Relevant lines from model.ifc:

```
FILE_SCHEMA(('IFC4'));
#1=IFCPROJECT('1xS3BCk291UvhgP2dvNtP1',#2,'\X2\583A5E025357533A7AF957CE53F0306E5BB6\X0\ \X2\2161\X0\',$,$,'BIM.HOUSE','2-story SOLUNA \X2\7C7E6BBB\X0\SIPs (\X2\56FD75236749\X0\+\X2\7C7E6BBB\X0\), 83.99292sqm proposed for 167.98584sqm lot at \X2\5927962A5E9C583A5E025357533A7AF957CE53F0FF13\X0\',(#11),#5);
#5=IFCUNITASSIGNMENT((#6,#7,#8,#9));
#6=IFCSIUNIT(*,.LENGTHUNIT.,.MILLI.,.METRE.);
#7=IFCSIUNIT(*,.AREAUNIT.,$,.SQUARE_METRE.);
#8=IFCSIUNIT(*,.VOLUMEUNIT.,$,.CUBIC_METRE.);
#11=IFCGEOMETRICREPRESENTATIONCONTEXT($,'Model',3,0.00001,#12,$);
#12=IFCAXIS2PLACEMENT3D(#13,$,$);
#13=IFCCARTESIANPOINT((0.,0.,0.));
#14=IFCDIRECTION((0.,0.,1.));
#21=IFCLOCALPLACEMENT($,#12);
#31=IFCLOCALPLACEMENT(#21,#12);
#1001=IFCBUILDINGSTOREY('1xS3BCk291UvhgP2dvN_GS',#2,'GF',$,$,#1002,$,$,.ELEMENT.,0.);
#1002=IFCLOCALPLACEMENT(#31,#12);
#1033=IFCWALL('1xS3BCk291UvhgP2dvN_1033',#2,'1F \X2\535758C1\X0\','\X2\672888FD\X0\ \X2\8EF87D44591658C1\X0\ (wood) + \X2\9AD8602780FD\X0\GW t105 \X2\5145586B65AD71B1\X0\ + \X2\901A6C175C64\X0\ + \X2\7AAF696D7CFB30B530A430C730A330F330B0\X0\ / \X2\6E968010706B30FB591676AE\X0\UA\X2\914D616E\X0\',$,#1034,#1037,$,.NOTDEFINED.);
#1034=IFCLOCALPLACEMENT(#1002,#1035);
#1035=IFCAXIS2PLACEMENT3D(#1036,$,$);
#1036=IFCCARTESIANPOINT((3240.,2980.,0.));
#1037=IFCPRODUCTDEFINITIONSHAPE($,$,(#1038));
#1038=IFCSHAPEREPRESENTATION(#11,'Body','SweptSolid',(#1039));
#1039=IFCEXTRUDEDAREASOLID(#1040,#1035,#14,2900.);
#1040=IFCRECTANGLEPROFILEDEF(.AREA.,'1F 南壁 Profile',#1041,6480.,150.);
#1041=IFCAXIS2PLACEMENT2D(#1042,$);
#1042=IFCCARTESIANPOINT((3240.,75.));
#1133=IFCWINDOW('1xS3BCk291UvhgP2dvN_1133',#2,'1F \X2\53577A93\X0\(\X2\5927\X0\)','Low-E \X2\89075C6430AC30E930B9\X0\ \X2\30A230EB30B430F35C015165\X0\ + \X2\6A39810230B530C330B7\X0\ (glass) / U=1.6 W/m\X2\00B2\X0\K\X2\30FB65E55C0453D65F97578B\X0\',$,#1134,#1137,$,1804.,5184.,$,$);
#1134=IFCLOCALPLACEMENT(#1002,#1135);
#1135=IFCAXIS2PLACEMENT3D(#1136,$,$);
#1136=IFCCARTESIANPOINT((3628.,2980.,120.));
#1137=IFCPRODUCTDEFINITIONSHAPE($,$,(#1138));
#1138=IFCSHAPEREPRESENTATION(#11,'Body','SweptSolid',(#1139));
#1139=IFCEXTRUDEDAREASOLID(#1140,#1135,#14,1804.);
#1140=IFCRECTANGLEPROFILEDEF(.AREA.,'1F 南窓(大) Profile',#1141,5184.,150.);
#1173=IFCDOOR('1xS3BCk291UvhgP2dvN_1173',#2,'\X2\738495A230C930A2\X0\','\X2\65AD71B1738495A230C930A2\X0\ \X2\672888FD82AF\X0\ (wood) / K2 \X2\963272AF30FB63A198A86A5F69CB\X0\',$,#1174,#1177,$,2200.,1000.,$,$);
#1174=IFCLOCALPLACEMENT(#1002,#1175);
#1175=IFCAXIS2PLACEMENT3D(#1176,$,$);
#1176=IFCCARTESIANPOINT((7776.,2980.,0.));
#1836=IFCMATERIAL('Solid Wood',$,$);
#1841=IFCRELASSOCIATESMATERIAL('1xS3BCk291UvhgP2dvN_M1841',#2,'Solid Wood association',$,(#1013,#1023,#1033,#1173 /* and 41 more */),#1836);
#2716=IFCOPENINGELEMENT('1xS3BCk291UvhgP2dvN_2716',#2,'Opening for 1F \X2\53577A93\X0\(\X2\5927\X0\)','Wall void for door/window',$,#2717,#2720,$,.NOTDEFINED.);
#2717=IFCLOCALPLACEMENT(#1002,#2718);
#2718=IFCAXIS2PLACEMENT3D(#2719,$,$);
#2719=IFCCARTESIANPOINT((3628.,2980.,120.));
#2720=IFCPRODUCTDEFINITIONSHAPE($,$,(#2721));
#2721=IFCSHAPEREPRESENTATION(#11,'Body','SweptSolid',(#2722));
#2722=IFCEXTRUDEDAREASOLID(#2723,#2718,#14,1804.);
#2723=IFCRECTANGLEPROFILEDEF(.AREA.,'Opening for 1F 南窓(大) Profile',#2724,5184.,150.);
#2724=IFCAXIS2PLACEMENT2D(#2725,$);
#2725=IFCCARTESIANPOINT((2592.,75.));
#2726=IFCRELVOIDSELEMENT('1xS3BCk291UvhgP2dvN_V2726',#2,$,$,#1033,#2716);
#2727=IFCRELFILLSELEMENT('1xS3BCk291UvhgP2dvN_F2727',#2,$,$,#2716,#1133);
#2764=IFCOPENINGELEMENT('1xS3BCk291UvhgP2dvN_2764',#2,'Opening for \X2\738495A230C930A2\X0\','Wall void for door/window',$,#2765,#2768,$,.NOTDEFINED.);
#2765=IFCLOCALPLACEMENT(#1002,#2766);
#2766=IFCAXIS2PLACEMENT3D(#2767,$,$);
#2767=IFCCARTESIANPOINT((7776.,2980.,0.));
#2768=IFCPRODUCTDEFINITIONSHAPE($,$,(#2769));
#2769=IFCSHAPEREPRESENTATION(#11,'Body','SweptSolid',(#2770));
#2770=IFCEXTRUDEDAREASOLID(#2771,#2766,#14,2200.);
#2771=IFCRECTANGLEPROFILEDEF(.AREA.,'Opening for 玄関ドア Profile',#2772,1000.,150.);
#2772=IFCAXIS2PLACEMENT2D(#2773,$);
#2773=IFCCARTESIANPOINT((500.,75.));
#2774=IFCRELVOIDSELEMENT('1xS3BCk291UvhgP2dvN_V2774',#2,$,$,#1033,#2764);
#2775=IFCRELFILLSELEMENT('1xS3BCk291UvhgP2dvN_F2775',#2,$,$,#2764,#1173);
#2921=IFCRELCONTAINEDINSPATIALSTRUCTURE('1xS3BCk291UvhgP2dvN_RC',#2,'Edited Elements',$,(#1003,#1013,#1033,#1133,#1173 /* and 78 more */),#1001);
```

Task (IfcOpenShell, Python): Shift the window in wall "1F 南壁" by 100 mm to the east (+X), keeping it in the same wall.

```python
import ifcopenshell
import ifcopenshell.api.geometry
import ifcopenshell.util.placement

model = ifcopenshell.open("model.ifc")

window = model.by_guid("1xS3BCk291UvhgP2dvN_1133")
opening = window.FillsVoids[0].RelatingOpeningElement
wall = opening.VoidsElements[0].RelatingBuildingElement

wall_matrix = ifcopenshell.util.placement.get_local_placement(wall.ObjectPlacement)
shift = wall_matrix[:3, 0] * 100.0
before = ifcopenshell.util.placement.get_local_placement(window.ObjectPlacement)[:3, 3].copy()

# The window is not placed relative to its opening, so move both.
for product in (opening, window):
    matrix = ifcopenshell.util.placement.get_local_placement(product.ObjectPlacement)
    matrix[:3, 3] += shift
    ifcopenshell.api.geometry.edit_object_placement(model, product=product, matrix=matrix, is_si=False)

after = ifcopenshell.util.placement.get_local_placement(window.ObjectPlacement)[:3, 3]
print("window moved by", (after - before).round(3) + 0.0)

model.write("model_rev.ifc")
```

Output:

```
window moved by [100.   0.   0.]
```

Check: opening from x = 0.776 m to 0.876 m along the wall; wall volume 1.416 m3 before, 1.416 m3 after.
